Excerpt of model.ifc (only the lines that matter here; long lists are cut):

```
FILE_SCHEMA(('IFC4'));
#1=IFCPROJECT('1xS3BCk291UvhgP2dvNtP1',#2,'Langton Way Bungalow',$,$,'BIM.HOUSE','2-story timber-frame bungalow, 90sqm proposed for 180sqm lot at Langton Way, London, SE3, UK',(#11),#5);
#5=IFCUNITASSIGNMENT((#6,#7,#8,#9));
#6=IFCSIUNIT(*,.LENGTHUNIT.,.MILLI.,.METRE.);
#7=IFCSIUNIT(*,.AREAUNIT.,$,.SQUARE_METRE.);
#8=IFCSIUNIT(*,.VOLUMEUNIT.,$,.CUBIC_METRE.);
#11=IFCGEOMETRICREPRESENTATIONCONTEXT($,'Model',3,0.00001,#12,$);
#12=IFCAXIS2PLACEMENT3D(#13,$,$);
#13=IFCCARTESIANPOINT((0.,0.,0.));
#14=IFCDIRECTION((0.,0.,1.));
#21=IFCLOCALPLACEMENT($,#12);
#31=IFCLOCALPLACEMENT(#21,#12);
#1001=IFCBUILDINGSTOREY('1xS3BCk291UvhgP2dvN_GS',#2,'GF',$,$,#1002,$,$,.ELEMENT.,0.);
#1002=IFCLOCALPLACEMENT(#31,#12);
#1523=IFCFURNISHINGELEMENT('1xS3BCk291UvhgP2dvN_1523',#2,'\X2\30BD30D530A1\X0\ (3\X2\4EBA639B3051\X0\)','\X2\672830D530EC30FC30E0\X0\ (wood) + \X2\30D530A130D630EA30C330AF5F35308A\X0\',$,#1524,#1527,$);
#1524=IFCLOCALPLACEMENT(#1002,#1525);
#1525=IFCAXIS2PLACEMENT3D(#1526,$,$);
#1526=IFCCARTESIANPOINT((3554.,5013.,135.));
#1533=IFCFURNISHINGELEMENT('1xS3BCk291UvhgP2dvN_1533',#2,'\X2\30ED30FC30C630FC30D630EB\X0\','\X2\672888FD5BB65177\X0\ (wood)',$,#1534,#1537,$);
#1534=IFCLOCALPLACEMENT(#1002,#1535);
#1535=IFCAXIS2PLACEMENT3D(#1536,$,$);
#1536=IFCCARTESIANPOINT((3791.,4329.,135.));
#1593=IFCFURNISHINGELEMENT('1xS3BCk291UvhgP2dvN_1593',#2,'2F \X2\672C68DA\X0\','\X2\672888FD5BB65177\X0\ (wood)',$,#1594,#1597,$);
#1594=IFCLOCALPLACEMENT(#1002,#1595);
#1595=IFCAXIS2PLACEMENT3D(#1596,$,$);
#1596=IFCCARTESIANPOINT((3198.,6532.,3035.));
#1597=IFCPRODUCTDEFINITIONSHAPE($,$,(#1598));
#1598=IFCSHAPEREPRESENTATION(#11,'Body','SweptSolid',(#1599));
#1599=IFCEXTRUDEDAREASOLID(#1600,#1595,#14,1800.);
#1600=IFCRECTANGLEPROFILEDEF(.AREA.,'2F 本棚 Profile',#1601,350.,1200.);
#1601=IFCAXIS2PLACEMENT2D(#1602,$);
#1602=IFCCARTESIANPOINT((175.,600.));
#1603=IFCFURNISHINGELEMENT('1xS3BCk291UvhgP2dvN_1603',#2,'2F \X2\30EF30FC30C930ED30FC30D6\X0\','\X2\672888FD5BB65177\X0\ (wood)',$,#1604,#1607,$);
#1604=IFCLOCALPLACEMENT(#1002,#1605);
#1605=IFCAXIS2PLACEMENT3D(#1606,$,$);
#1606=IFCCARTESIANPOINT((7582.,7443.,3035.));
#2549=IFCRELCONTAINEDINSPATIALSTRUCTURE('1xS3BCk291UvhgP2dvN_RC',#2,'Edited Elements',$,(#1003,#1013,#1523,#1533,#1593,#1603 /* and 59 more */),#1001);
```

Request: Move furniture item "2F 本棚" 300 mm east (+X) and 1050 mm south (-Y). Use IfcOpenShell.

```python
import ifcopenshell
import ifcopenshell.api.geometry
import ifcopenshell.util.placement
import ifcopenshell.util.unit

model = ifcopenshell.open("model.ifc")
unit_scale = ifcopenshell.util.unit.calculate_unit_scale(model)

item = model.by_guid("1xS3BCk291UvhgP2dvN_1593")
matrix = ifcopenshell.util.placement.get_local_placement(item.ObjectPlacement)
matrix[0, 3] += 0.3 / unit_scale
matrix[1, 3] -= 1.05 / unit_scale
ifcopenshell.api.geometry.edit_object_placement(model, product=item, matrix=matrix, is_si=False)

print(ifcopenshell.util.placement.get_local_placement(item.ObjectPlacement).round(3) + 0.0)

model.write("model-out.ifc")
```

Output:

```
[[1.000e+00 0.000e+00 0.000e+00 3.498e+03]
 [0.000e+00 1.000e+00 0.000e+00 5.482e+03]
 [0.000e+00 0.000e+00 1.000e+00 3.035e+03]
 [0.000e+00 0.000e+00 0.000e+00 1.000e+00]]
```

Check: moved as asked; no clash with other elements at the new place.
